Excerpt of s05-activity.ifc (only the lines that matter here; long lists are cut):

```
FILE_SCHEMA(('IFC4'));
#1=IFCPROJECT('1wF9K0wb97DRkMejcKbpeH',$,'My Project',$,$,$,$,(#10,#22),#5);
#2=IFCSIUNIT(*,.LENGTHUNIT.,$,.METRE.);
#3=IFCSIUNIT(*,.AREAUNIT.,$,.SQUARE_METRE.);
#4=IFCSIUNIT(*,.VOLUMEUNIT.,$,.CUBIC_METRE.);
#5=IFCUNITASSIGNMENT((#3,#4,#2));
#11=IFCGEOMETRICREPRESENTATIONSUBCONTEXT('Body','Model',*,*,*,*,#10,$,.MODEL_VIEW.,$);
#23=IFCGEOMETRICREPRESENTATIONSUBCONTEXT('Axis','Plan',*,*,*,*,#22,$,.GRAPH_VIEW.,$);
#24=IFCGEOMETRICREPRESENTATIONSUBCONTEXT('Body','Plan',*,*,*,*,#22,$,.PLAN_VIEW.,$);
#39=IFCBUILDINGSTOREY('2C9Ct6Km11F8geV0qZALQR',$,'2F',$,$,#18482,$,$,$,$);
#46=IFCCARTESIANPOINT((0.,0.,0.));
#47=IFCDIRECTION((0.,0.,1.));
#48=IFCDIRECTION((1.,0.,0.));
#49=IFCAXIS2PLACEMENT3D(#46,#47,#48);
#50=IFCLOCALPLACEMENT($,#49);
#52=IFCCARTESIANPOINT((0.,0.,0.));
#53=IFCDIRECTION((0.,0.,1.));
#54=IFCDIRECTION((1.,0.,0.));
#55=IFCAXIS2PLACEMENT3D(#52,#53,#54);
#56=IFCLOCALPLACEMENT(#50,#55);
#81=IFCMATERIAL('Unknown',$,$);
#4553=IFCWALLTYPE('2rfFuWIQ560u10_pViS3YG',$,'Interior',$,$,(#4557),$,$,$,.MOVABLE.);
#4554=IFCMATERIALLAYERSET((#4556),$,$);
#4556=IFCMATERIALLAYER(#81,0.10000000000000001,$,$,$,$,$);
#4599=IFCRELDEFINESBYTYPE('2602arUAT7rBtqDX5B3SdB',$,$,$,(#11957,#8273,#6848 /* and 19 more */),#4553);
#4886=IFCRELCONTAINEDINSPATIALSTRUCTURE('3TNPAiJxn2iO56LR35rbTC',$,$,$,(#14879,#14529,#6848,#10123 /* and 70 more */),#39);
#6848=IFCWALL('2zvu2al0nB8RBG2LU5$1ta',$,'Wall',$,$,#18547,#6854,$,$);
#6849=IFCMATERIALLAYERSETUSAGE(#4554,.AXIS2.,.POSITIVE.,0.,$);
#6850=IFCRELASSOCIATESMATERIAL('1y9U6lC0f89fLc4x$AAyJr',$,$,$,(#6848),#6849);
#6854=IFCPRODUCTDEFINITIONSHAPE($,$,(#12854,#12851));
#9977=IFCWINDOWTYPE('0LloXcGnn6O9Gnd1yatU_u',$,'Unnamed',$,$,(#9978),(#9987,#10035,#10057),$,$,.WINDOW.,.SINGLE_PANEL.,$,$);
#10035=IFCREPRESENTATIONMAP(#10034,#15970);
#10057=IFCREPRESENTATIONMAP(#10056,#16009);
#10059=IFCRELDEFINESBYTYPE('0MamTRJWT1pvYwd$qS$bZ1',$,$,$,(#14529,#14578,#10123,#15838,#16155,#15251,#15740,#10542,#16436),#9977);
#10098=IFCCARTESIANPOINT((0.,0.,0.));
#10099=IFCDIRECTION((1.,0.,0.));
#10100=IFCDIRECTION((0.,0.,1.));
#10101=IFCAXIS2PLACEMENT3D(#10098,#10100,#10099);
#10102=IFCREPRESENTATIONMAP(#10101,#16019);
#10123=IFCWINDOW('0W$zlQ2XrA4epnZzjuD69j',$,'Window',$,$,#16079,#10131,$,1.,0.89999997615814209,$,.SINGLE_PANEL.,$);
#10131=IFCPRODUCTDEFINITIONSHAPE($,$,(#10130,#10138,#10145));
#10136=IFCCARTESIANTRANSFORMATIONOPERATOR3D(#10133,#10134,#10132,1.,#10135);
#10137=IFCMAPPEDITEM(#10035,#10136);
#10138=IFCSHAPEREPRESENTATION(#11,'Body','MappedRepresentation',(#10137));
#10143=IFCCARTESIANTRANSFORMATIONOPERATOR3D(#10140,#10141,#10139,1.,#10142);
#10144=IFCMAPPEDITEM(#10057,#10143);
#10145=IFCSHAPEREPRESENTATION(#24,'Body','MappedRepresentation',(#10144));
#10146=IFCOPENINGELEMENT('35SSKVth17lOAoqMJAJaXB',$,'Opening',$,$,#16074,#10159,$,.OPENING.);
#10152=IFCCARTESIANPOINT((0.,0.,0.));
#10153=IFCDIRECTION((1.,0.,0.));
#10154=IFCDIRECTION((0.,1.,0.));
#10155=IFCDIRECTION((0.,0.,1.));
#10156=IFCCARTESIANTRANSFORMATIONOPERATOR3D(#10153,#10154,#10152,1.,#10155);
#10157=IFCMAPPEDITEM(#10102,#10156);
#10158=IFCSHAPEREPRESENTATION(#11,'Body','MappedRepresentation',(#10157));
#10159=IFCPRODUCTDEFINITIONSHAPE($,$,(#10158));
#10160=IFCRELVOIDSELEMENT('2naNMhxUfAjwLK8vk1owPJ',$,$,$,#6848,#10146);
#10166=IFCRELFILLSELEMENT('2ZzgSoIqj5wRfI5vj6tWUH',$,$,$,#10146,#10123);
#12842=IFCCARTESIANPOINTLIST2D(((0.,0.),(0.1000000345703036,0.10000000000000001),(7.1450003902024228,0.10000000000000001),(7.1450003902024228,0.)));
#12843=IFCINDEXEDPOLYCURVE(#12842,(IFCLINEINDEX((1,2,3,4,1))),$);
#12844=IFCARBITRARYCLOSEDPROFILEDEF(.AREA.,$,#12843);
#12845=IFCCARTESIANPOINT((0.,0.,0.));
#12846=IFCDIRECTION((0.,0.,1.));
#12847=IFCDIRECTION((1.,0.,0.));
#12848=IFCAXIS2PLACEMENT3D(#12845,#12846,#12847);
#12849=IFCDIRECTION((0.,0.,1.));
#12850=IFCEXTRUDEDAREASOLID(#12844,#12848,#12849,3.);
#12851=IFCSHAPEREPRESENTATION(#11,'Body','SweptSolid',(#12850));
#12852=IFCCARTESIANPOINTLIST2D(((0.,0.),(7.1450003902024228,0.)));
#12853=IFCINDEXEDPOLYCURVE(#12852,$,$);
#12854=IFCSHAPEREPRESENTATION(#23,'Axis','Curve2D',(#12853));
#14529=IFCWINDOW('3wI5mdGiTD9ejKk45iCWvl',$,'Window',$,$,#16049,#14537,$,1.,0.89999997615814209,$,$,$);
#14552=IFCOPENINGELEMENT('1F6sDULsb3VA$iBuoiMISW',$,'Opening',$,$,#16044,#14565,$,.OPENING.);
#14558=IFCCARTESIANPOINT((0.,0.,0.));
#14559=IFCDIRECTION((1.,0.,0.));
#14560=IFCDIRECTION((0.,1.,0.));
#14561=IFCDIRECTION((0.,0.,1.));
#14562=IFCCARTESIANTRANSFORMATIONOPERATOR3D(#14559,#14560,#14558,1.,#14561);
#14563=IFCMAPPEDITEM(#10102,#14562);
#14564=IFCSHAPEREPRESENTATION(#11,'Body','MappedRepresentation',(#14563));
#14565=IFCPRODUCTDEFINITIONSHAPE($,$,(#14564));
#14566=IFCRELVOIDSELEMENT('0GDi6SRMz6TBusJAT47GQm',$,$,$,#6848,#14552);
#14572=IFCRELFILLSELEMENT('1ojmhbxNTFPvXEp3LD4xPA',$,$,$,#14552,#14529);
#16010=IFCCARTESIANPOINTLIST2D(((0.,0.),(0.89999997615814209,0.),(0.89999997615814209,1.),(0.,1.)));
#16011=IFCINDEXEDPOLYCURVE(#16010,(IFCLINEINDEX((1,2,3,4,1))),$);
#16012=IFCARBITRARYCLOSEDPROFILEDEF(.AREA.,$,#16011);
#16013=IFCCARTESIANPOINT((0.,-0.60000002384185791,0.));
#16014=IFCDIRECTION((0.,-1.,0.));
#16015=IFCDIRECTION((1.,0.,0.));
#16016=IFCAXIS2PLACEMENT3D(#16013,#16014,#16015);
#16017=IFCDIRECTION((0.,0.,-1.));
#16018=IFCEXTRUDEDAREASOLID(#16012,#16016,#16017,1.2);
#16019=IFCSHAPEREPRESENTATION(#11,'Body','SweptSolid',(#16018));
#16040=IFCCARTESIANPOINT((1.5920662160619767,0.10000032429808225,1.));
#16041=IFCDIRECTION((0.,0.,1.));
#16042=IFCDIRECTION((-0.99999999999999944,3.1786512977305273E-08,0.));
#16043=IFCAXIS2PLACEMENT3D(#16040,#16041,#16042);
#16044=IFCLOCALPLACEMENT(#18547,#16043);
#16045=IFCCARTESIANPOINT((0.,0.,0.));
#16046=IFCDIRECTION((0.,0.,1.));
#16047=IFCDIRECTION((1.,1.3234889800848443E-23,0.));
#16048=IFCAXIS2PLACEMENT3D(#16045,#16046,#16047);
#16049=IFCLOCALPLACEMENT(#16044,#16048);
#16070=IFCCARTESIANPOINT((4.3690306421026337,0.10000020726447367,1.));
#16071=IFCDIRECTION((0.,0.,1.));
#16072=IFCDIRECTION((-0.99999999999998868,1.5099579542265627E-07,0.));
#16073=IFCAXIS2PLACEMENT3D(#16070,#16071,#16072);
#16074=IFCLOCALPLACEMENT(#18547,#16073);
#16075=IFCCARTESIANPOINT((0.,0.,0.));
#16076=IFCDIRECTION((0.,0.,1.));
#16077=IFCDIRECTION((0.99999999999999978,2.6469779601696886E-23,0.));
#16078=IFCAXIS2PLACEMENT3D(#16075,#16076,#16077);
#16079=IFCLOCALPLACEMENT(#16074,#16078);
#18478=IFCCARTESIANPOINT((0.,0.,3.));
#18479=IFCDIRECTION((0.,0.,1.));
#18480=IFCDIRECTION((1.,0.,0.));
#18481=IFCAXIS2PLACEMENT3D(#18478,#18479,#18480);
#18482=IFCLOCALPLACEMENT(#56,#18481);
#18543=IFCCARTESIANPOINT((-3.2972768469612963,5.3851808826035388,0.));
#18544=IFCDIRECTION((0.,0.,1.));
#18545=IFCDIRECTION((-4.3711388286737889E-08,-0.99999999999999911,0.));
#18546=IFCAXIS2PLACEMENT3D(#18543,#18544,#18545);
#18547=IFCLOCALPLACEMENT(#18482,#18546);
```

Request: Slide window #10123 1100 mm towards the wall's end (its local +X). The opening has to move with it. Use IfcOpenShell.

```python
import ifcopenshell
import ifcopenshell.api.geometry
import ifcopenshell.util.placement
import ifcopenshell.util.unit

model = ifcopenshell.open("s05-activity.ifc")
unit_scale = ifcopenshell.util.unit.calculate_unit_scale(model)

window = model.by_guid("0W$zlQ2XrA4epnZzjuD69j")
opening = window.FillsVoids[0].RelatingOpeningElement
wall = opening.VoidsElements[0].RelatingBuildingElement

wall_matrix = ifcopenshell.util.placement.get_local_placement(wall.ObjectPlacement)
shift = wall_matrix[:3, 0] * 1.1 / unit_scale
before = ifcopenshell.util.placement.get_local_placement(window.ObjectPlacement)[:3, 3].copy()

# The window is placed relative to its opening, so it follows when the opening moves.
matrix = ifcopenshell.util.placement.get_local_placement(opening.ObjectPlacement)
matrix[:3, 3] += shift
ifcopenshell.api.geometry.edit_object_placement(
    model, product=opening, matrix=matrix, is_si=False, should_transform_children=True
)

after = ifcopenshell.util.placement.get_local_placement(window.ObjectPlacement)[:3, 3]
print("window moved by", (after - before).round(3) + 0.0)

model.write("s05-activity_edited.ifc")
```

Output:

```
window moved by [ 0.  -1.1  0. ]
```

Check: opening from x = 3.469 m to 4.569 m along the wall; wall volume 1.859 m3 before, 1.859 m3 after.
